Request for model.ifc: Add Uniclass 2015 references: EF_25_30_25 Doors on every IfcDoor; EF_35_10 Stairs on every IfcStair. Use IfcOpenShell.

First a look at what the model holds.

```python
import ifcopenshell

model = ifcopenshell.open("model.ifc")
print(model.schema)
print("classifications:", [c.Name for c in model.by_type("IfcClassification")])
for ifc_class in ("IfcDoor", "IfcRoof", "IfcStair", "IfcWall", "IfcWindow"):
    print(ifc_class, len(model.by_type(ifc_class)))
```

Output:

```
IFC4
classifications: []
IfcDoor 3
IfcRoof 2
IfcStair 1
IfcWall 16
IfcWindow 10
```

```python
import ifcopenshell
import ifcopenshell.api.classification

model = ifcopenshell.open("model.ifc")

system = ifcopenshell.api.classification.add_classification(model, classification="Uniclass 2015")

codes = {
    "IfcDoor": ("EF_25_30_25", "Doors"),
    "IfcStair": ("EF_35_10", "Stairs"),
}
for ifc_class, (code, name) in codes.items():
    products = model.by_type(ifc_class)
    ifcopenshell.api.classification.add_reference(
        model, products=products, classification=system, identification=code, name=name
    )
    print(code, len(products))

model.write("model_v2.ifc")
```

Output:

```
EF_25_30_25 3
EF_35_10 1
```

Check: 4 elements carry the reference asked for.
